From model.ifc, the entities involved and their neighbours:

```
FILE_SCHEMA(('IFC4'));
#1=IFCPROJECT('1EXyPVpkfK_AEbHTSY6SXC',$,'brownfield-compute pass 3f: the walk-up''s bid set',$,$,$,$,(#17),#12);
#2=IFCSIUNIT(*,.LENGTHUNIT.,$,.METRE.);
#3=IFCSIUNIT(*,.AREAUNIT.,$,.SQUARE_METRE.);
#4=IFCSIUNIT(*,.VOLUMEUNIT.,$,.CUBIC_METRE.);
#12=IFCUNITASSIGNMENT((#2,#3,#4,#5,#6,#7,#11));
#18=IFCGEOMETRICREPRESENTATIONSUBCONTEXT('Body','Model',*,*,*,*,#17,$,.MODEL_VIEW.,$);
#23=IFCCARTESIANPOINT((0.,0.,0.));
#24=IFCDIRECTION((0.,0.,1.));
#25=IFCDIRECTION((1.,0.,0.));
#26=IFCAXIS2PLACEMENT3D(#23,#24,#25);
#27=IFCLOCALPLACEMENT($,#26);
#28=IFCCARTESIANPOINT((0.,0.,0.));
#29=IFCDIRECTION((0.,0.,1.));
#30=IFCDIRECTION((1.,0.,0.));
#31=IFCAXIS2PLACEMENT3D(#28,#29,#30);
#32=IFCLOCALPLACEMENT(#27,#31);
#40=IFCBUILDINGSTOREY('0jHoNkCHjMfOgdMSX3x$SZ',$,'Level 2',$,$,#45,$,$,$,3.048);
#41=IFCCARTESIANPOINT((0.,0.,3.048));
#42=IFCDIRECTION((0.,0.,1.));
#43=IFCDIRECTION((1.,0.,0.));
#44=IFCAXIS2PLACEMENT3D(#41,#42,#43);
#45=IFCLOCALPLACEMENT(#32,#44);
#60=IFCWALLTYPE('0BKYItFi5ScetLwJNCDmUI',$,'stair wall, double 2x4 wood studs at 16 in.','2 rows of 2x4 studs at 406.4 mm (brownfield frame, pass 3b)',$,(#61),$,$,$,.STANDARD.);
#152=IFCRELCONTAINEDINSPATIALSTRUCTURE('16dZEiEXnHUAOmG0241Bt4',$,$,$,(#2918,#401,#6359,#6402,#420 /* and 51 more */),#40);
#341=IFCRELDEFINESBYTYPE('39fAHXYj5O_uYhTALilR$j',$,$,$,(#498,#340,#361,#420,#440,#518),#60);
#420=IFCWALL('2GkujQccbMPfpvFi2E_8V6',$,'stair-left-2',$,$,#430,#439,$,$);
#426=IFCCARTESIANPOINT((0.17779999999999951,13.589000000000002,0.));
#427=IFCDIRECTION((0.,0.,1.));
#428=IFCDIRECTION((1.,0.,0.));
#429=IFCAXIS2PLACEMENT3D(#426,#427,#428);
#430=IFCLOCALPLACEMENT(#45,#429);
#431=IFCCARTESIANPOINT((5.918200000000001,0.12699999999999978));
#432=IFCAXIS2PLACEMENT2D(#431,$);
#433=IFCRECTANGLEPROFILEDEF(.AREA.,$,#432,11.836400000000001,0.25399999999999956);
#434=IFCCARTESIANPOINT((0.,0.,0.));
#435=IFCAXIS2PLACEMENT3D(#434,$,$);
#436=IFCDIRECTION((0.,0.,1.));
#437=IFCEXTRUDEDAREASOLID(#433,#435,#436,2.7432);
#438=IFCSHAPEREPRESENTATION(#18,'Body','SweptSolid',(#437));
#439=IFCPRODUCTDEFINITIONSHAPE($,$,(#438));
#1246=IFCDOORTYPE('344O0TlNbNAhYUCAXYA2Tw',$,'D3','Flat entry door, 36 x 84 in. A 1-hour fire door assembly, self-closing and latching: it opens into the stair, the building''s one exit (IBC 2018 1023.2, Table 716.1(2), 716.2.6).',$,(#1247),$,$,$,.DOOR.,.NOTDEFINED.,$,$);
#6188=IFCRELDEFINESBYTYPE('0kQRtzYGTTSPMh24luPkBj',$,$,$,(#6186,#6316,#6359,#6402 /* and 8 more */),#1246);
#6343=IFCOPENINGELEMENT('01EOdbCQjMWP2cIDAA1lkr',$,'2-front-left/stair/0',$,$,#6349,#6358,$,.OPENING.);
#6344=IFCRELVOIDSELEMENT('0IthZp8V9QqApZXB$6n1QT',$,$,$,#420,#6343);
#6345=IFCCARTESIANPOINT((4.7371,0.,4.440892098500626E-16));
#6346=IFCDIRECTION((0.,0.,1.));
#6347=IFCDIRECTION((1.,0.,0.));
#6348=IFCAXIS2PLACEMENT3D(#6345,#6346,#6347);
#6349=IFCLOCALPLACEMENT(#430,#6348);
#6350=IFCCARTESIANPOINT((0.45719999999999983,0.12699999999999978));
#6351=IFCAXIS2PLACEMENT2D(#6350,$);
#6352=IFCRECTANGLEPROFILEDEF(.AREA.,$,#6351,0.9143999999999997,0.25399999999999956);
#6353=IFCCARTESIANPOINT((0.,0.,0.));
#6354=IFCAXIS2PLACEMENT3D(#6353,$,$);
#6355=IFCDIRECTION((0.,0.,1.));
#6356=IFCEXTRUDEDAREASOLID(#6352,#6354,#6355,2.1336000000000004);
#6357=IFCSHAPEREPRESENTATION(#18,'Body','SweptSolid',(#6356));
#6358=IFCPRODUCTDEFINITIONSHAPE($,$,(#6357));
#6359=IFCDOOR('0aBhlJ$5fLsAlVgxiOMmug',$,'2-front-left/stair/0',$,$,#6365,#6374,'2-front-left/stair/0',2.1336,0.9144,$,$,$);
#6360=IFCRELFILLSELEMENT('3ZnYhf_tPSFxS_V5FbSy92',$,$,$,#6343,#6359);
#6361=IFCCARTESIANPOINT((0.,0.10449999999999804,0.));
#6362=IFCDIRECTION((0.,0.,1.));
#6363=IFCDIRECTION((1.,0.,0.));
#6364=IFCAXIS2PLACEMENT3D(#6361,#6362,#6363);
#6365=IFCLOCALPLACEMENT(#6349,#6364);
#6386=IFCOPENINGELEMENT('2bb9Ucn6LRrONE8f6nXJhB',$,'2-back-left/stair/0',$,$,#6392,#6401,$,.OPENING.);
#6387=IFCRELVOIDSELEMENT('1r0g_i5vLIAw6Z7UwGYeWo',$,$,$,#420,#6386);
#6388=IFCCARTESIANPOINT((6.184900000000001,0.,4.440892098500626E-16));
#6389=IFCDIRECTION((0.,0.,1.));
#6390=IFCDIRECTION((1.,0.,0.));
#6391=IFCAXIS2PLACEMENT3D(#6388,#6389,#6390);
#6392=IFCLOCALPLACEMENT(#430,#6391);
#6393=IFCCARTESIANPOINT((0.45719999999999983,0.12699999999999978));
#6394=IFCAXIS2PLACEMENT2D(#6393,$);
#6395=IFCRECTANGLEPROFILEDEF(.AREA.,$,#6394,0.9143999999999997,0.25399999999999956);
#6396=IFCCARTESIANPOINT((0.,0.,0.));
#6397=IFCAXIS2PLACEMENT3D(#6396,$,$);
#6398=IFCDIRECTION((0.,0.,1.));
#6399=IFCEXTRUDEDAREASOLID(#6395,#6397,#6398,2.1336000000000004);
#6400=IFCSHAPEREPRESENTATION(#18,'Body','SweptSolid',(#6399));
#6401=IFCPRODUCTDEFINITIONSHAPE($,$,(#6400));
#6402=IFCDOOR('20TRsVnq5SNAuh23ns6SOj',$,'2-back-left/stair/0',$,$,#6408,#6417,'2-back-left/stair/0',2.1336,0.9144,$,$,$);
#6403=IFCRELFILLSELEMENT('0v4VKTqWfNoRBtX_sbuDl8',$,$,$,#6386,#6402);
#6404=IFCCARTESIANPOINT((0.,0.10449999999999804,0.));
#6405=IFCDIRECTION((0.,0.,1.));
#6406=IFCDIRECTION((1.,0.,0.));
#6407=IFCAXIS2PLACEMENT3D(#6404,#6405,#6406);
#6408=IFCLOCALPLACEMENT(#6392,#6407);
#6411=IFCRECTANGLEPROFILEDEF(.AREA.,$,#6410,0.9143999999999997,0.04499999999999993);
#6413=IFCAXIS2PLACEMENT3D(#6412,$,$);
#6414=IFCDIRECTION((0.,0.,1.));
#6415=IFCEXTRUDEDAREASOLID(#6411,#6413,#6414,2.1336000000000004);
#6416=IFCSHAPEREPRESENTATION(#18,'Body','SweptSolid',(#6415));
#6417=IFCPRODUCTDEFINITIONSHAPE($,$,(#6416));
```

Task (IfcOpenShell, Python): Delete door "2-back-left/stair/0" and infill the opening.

```python
import ifcopenshell
import ifcopenshell.api.feature
import ifcopenshell.api.root
import ifcopenshell.geom
import ifcopenshell.util.shape

model = ifcopenshell.open("model.ifc")
settings = ifcopenshell.geom.settings()


def volume(element):
    """Net volume in cubic metres, openings subtracted."""
    shape = ifcopenshell.geom.create_shape(settings, element)
    return ifcopenshell.util.shape.get_volume(shape.geometry)


door = model.by_guid("20TRsVnq5SNAuh23ns6SOj")
opening = door.FillsVoids[0].RelatingOpeningElement
wall = opening.VoidsElements[0].RelatingBuildingElement
before = volume(wall)

ifcopenshell.api.root.remove_product(model, product=door)
ifcopenshell.api.feature.remove_feature(model, feature=opening)

after = volume(wall)

print(f"wall volume {before:.3f} -> {after:.3f} m3")

model.write("model_edited.ifc")
```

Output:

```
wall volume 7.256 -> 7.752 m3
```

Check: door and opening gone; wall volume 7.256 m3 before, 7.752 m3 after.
